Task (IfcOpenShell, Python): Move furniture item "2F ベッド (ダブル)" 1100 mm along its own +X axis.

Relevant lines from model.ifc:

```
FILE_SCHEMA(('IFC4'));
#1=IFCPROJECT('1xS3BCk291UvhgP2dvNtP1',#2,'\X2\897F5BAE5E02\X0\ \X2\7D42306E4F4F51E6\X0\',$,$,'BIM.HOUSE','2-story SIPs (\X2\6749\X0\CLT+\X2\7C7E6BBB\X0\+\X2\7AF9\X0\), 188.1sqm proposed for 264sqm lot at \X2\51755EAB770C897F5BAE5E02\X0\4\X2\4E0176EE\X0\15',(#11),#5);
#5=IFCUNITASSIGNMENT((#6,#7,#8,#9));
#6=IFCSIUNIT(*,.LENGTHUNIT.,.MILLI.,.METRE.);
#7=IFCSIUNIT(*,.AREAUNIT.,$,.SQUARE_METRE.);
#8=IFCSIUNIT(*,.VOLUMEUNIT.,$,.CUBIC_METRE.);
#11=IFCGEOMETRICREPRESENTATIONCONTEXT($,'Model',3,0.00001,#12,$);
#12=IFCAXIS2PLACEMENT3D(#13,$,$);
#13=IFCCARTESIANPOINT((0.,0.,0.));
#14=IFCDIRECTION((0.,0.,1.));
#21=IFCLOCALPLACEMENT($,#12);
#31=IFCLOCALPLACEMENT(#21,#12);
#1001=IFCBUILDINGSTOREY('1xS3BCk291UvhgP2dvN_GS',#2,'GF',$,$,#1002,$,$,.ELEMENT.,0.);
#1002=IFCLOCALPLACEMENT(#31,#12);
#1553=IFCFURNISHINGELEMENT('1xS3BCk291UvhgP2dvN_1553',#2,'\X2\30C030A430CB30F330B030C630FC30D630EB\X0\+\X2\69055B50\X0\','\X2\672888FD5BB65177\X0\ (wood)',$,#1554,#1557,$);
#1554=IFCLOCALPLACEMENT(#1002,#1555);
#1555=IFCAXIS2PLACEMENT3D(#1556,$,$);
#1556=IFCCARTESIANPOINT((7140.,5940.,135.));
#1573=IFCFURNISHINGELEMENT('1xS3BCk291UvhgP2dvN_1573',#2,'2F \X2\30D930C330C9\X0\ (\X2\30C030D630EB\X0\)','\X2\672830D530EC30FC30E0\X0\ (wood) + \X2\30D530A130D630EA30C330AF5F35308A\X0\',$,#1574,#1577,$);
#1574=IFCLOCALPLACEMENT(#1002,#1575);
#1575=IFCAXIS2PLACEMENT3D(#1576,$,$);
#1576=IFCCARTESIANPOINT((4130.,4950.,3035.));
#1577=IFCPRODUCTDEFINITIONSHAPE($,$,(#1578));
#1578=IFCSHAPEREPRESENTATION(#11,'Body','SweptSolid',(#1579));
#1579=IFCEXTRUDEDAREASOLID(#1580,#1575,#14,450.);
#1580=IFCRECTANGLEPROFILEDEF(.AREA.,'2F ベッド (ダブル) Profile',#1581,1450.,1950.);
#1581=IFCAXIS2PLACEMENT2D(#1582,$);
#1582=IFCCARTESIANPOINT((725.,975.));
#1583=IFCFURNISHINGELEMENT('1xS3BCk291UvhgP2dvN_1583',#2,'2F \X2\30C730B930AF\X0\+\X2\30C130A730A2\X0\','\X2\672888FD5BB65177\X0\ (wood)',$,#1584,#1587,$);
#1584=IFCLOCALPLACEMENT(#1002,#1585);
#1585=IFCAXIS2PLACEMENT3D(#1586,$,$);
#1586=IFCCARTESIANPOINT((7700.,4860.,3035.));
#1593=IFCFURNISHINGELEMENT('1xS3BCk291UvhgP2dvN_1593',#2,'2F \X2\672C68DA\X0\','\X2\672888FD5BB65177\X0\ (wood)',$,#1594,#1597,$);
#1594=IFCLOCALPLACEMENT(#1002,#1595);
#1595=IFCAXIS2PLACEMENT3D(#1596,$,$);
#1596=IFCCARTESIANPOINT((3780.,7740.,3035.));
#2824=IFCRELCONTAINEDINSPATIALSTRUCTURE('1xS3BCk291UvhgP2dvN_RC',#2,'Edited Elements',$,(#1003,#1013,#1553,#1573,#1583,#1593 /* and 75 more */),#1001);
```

```python
import ifcopenshell
import ifcopenshell.api.geometry
import ifcopenshell.util.placement

model = ifcopenshell.open("model.ifc")

item = model.by_guid("1xS3BCk291UvhgP2dvN_1573")
matrix = ifcopenshell.util.placement.get_local_placement(item.ObjectPlacement)
matrix[:3, 3] += matrix[:3, 0] * 1100.0
ifcopenshell.api.geometry.edit_object_placement(model, product=item, matrix=matrix, is_si=False)

print(ifcopenshell.util.placement.get_local_placement(item.ObjectPlacement).round(3) + 0.0)

model.write("model_rev.ifc")
```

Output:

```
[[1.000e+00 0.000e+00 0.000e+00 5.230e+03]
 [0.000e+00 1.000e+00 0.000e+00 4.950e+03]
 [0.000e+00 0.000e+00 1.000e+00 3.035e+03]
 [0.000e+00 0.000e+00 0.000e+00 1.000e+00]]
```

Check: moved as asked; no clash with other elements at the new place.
